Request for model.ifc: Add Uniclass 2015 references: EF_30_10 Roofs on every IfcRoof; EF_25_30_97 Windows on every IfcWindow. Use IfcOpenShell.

First a look at what the model holds.

```python
import ifcopenshell

model = ifcopenshell.open("model.ifc")
print(model.schema)
print("classifications:", [c.Name for c in model.by_type("IfcClassification")])
for ifc_class in ("IfcDoor", "IfcRoof", "IfcStair", "IfcWall", "IfcWindow"):
    print(ifc_class, len(model.by_type(ifc_class)))
```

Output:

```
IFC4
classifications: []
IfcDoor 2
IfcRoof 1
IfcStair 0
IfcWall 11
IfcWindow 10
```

```python
import ifcopenshell
import ifcopenshell.api.classification

model = ifcopenshell.open("model.ifc")

system = ifcopenshell.api.classification.add_classification(model, classification="Uniclass 2015")

codes = {
    "IfcRoof": ("EF_30_10", "Roofs"),
    "IfcWindow": ("EF_25_30_97", "Windows"),
}
for ifc_class, (code, name) in codes.items():
    products = model.by_type(ifc_class)
    ifcopenshell.api.classification.add_reference(
        model, products=products, classification=system, identification=code, name=name
    )
    print(code, len(products))

model.write("model_v2.ifc")
```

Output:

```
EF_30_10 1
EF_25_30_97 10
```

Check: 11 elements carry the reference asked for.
